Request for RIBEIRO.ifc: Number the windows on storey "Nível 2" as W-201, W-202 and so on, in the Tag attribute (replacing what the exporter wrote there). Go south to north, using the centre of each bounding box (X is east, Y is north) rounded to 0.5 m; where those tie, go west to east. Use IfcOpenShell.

First a look at what the model holds.

```python
import ifcopenshell
import ifcopenshell.util.element
import ifcopenshell.util.placement

model = ifcopenshell.open("RIBEIRO.ifc")
print(model.schema)
storey = next(s for s in model.by_type("IfcBuildingStorey") if s.Name == "Nível 2")
windows = [e for e in ifcopenshell.util.element.get_decomposition(storey) if e.is_a("IfcWindow")]
for e in sorted(windows, key=lambda e: e.id()):
    origin = ifcopenshell.util.placement.get_local_placement(e.ObjectPlacement)[:3, 3]
    print(e.id(), e.Tag, e.Name, origin.round(2) + 0.0, sep=" | ")
```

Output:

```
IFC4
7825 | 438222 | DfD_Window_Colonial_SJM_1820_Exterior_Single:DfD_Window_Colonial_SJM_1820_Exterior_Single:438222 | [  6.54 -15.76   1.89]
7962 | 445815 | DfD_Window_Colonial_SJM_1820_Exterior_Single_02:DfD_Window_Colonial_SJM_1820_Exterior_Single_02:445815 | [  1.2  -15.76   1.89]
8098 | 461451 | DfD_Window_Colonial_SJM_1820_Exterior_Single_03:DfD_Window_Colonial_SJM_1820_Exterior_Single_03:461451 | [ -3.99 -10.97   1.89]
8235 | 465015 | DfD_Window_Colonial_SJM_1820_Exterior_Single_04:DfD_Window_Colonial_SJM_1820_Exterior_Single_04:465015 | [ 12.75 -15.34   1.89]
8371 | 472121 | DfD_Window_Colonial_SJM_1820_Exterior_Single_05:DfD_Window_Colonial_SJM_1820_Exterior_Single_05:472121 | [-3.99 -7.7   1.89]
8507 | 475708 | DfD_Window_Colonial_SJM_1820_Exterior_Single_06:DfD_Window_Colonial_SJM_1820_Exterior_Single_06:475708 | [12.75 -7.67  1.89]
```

```python
import ifcopenshell
import ifcopenshell.geom
import ifcopenshell.util.element
import ifcopenshell.util.shape

model = ifcopenshell.open("RIBEIRO.ifc")
settings = ifcopenshell.geom.settings()
settings.set("use-world-coords", True)


def centre(element):
    shape = ifcopenshell.geom.create_shape(settings, element)
    return ifcopenshell.util.shape.get_bbox_centroid(shape.geometry)


storey = next(s for s in model.by_type("IfcBuildingStorey") if s.Name == "Nível 2")
windows = [e for e in ifcopenshell.util.element.get_decomposition(storey) if e.is_a("IfcWindow")]

# Insertion points can sit at a corner or the storey origin, so sort by the geometry (in metres).
centres = {e: centre(e) for e in windows}
windows.sort(key=lambda e: (round(centres[e][1] / 0.5), centres[e][0]))

for i, e in enumerate(windows, start=1):
    number = f"W-2{i:02d}"
    e.Tag = number
    print(e.id(), number)

model.write("RIBEIRO_edited.ifc")
```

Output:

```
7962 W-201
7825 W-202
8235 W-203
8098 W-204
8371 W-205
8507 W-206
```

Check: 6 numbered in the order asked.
